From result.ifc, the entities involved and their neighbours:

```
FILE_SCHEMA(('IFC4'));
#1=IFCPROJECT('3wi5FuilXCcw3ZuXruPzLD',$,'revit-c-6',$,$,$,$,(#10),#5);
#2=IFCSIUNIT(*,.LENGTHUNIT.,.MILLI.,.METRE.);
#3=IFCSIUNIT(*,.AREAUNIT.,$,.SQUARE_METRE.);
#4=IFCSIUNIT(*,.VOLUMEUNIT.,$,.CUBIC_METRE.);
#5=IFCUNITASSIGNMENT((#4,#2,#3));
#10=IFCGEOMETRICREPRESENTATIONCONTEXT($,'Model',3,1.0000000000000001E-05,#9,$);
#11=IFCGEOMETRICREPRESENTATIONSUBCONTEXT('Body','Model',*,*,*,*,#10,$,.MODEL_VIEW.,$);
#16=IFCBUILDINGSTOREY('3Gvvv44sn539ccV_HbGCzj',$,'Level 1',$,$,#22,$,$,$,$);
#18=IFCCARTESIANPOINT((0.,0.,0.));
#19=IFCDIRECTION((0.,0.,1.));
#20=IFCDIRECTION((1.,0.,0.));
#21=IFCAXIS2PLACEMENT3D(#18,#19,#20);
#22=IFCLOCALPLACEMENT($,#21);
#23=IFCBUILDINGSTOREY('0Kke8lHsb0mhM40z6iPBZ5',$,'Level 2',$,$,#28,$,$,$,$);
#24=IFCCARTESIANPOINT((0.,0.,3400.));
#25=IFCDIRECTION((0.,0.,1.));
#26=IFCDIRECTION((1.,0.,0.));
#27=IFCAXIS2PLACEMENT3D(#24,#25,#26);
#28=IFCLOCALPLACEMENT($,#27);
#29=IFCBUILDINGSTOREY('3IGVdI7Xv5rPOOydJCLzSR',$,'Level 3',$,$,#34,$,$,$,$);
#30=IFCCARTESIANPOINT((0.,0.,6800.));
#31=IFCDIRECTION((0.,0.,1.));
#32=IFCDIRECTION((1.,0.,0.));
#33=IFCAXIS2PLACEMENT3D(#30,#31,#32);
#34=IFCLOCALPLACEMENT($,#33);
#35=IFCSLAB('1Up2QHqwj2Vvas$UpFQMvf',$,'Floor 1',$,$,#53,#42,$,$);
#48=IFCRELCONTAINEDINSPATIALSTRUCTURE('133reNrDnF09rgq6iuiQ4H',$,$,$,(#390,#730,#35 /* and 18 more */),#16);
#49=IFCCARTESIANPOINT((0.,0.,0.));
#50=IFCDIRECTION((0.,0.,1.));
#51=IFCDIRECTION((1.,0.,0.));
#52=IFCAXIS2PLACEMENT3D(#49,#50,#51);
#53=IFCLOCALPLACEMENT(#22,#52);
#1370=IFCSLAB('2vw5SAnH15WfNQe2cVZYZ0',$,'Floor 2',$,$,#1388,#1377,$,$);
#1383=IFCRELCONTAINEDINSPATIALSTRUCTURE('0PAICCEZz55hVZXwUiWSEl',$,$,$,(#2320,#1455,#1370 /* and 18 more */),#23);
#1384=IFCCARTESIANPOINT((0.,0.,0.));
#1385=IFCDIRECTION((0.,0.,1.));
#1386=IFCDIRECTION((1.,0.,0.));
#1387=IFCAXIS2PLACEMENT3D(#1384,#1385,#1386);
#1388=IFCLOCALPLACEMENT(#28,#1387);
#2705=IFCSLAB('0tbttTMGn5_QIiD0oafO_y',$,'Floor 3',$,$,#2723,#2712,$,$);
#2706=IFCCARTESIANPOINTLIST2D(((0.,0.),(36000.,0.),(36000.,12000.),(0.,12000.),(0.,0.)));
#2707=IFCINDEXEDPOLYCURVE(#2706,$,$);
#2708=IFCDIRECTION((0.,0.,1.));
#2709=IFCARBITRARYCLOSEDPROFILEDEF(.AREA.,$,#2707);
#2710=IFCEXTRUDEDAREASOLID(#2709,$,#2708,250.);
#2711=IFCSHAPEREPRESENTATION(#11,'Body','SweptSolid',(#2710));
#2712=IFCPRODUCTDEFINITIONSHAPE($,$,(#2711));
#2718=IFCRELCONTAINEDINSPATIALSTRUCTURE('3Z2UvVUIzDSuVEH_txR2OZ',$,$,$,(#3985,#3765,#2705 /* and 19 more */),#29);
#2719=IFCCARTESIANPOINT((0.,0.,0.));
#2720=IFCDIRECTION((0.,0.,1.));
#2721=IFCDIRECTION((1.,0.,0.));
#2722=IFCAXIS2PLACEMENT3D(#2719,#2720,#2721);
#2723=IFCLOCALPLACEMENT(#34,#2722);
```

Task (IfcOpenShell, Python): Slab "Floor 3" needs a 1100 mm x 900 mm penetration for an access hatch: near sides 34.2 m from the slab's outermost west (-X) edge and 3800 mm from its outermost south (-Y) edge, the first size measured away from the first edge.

```python
import numpy as np
import ifcopenshell
import ifcopenshell.api.feature
import ifcopenshell.api.geometry
import ifcopenshell.api.root
import ifcopenshell.geom
import ifcopenshell.util.placement
import ifcopenshell.util.representation
import ifcopenshell.util.shape
import ifcopenshell.util.unit

model = ifcopenshell.open("result.ifc")
unit_scale = ifcopenshell.util.unit.calculate_unit_scale(model)
settings = ifcopenshell.geom.settings()


def volume(element):
    """Net volume in cubic metres, openings subtracted."""
    shape = ifcopenshell.geom.create_shape(settings, element)
    return ifcopenshell.util.shape.get_volume(shape.geometry)


slab = model.by_guid("0tbttTMGn5_QIiD0oafO_y")
before = volume(slab)

# Extent in the slab's own axes, in metres. The edges named are its -X and -Y sides.
slab_shape = ifcopenshell.geom.create_shape(settings, slab)
vertices = ifcopenshell.util.shape.get_vertices(slab_shape.geometry)
x_min, y_min, bottom = vertices.min(axis=0)
top = vertices[:, 2].max()

opening = ifcopenshell.api.root.create_entity(model, ifc_class="IfcOpeningElement", name="Access hatch opening", predefined_type="OPENING")
context = ifcopenshell.util.representation.get_context(model, "Model", "Body", "MODEL_VIEW")
width, depth = 1.1, 0.9
outline = [(0.0, 0.0), (width, 0.0), (width, depth), (0.0, depth), (0.0, 0.0)]
# Overshoot both faces by 50 mm so the cut is clean.
shape = ifcopenshell.api.geometry.add_slab_representation(
    model, context=context, depth=top - bottom + 0.1, polyline=outline
)
ifcopenshell.api.geometry.assign_representation(model, product=opening, representation=shape)

matrix = ifcopenshell.util.placement.get_local_placement(slab.ObjectPlacement)
matrix[:, 3] = matrix @ np.append(np.array([x_min + 34.2, y_min + 3.8, bottom - 0.05]) / unit_scale, 1.0)
ifcopenshell.api.geometry.edit_object_placement(model, product=opening, matrix=matrix, is_si=False)
ifcopenshell.api.feature.add_feature(model, feature=opening, element=slab)

after = volume(slab)

print(f"slab volume {before:.3f} -> {after:.3f} m3")

model.write("result_v2.ifc")
```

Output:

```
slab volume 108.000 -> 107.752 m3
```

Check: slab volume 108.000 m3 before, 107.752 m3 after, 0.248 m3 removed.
